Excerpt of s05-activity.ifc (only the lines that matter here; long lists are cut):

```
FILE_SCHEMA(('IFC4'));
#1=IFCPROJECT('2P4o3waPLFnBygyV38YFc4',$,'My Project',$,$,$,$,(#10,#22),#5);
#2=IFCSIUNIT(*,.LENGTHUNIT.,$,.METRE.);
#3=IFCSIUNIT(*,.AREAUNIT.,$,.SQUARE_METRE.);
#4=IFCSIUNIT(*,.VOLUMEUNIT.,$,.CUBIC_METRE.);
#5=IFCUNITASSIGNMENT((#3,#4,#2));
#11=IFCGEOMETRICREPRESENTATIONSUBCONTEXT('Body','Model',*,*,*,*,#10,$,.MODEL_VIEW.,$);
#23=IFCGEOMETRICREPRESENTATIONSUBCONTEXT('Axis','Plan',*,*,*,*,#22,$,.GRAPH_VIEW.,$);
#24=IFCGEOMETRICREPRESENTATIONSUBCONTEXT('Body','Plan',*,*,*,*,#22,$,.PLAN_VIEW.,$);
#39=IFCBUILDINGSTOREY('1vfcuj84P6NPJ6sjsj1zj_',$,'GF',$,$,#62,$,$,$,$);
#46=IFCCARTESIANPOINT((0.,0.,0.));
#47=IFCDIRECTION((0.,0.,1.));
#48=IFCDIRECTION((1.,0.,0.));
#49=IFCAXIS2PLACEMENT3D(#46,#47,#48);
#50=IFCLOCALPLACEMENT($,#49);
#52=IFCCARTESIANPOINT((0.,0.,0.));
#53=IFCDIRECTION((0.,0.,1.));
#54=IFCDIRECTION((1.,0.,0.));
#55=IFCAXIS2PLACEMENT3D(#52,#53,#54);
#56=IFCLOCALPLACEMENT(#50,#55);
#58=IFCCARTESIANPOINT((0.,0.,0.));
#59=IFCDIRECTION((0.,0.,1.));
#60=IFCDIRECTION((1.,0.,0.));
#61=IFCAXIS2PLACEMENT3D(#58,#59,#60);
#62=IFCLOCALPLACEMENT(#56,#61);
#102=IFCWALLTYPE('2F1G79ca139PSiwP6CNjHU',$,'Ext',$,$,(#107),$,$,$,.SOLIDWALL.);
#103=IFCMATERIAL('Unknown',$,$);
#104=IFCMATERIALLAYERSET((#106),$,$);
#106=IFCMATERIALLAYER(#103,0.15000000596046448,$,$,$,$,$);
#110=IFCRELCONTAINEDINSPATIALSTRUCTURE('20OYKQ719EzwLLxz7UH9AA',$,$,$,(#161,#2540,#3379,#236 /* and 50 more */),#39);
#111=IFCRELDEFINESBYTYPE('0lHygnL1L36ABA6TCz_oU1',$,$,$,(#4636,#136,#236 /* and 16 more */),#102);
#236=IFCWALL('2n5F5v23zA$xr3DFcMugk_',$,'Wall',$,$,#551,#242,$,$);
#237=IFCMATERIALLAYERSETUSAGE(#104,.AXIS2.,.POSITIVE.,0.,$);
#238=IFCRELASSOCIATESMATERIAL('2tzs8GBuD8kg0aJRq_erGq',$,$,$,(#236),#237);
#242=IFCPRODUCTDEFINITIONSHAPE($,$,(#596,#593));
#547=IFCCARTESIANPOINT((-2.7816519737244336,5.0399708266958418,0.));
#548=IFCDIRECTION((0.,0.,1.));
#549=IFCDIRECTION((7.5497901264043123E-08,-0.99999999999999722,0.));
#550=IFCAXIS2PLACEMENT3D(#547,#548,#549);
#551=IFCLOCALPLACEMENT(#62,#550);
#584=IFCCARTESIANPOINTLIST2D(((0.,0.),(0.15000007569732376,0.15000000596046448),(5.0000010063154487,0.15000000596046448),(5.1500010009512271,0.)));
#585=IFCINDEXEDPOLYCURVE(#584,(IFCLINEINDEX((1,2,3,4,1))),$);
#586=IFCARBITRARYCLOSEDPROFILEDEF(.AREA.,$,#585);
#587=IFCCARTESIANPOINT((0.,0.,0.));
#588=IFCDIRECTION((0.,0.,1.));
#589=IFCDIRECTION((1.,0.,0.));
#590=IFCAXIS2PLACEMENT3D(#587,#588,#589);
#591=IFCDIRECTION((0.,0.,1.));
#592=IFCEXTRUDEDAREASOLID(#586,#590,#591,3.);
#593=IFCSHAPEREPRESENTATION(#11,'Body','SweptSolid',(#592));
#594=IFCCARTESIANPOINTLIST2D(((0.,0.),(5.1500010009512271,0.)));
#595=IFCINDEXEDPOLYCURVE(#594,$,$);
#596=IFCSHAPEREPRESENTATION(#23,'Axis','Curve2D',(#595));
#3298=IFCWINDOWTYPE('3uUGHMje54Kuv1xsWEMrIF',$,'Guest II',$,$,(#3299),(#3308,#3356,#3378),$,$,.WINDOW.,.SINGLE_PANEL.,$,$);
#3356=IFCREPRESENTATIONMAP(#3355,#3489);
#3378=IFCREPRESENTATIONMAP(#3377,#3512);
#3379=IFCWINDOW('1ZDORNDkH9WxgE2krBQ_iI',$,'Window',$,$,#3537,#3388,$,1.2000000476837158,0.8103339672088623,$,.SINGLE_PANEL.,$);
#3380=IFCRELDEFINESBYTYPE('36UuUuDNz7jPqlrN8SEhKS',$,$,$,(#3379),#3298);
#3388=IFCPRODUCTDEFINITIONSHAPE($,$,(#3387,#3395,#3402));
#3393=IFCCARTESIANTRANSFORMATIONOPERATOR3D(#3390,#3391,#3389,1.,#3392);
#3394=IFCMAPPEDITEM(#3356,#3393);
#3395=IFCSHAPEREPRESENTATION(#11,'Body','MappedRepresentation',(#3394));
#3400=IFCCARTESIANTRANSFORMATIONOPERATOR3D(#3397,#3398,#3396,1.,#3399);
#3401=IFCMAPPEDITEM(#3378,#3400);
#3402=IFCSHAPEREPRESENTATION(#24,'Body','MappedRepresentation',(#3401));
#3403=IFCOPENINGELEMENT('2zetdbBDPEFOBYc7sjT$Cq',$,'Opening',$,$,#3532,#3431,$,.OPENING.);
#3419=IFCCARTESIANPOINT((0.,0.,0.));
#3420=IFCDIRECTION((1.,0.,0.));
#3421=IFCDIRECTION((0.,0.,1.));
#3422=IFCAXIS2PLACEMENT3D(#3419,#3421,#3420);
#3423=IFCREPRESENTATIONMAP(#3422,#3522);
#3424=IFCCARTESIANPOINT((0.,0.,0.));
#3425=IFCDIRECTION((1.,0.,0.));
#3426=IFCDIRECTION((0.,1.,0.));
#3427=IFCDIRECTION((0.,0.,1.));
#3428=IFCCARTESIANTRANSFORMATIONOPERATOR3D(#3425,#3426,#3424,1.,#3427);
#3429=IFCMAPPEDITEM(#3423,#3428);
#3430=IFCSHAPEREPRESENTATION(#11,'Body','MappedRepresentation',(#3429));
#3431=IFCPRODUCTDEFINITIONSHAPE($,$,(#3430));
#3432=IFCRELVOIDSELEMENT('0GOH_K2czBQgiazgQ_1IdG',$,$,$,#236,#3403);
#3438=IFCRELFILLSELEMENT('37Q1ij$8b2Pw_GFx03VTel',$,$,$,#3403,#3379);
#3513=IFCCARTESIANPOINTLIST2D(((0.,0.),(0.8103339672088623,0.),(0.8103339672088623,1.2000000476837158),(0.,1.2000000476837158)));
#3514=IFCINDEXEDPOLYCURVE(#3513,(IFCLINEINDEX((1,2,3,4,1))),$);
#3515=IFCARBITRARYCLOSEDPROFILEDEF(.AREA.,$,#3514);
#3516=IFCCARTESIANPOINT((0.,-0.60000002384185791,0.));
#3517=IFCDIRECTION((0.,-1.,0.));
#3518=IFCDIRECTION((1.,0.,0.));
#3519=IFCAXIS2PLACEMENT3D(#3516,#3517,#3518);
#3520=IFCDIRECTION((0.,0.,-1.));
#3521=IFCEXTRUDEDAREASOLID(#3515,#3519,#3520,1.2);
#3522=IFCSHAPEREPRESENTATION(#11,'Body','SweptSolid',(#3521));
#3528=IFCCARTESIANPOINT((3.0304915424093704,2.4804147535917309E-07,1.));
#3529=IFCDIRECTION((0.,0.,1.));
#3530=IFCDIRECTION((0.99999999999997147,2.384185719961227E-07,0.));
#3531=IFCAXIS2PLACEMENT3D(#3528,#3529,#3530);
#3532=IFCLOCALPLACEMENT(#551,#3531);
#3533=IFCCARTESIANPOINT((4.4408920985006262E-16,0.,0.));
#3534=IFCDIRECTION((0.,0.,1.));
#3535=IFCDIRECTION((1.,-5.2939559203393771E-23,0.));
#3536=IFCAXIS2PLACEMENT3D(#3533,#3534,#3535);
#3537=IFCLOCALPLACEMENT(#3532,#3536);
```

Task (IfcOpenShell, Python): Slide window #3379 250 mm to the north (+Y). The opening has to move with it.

```python
import ifcopenshell
import ifcopenshell.api.geometry
import ifcopenshell.util.placement
import ifcopenshell.util.unit

model = ifcopenshell.open("s05-activity.ifc")
unit_scale = ifcopenshell.util.unit.calculate_unit_scale(model)

window = model.by_guid("1ZDORNDkH9WxgE2krBQ_iI")
opening = window.FillsVoids[0].RelatingOpeningElement
wall = opening.VoidsElements[0].RelatingBuildingElement

wall_matrix = ifcopenshell.util.placement.get_local_placement(wall.ObjectPlacement)
shift = wall_matrix[:3, 0] * -0.25 / unit_scale
before = ifcopenshell.util.placement.get_local_placement(window.ObjectPlacement)[:3, 3].copy()

# The window is placed relative to its opening, so it follows when the opening moves.
matrix = ifcopenshell.util.placement.get_local_placement(opening.ObjectPlacement)
matrix[:3, 3] += shift
ifcopenshell.api.geometry.edit_object_placement(
    model, product=opening, matrix=matrix, is_si=False, should_transform_children=True
)

after = ifcopenshell.util.placement.get_local_placement(window.ObjectPlacement)[:3, 3]
print("window moved by", (after - before).round(3) + 0.0)

model.write("s05-activity-out.ifc")
```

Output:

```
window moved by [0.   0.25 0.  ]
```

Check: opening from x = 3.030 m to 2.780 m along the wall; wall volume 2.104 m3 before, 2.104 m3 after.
